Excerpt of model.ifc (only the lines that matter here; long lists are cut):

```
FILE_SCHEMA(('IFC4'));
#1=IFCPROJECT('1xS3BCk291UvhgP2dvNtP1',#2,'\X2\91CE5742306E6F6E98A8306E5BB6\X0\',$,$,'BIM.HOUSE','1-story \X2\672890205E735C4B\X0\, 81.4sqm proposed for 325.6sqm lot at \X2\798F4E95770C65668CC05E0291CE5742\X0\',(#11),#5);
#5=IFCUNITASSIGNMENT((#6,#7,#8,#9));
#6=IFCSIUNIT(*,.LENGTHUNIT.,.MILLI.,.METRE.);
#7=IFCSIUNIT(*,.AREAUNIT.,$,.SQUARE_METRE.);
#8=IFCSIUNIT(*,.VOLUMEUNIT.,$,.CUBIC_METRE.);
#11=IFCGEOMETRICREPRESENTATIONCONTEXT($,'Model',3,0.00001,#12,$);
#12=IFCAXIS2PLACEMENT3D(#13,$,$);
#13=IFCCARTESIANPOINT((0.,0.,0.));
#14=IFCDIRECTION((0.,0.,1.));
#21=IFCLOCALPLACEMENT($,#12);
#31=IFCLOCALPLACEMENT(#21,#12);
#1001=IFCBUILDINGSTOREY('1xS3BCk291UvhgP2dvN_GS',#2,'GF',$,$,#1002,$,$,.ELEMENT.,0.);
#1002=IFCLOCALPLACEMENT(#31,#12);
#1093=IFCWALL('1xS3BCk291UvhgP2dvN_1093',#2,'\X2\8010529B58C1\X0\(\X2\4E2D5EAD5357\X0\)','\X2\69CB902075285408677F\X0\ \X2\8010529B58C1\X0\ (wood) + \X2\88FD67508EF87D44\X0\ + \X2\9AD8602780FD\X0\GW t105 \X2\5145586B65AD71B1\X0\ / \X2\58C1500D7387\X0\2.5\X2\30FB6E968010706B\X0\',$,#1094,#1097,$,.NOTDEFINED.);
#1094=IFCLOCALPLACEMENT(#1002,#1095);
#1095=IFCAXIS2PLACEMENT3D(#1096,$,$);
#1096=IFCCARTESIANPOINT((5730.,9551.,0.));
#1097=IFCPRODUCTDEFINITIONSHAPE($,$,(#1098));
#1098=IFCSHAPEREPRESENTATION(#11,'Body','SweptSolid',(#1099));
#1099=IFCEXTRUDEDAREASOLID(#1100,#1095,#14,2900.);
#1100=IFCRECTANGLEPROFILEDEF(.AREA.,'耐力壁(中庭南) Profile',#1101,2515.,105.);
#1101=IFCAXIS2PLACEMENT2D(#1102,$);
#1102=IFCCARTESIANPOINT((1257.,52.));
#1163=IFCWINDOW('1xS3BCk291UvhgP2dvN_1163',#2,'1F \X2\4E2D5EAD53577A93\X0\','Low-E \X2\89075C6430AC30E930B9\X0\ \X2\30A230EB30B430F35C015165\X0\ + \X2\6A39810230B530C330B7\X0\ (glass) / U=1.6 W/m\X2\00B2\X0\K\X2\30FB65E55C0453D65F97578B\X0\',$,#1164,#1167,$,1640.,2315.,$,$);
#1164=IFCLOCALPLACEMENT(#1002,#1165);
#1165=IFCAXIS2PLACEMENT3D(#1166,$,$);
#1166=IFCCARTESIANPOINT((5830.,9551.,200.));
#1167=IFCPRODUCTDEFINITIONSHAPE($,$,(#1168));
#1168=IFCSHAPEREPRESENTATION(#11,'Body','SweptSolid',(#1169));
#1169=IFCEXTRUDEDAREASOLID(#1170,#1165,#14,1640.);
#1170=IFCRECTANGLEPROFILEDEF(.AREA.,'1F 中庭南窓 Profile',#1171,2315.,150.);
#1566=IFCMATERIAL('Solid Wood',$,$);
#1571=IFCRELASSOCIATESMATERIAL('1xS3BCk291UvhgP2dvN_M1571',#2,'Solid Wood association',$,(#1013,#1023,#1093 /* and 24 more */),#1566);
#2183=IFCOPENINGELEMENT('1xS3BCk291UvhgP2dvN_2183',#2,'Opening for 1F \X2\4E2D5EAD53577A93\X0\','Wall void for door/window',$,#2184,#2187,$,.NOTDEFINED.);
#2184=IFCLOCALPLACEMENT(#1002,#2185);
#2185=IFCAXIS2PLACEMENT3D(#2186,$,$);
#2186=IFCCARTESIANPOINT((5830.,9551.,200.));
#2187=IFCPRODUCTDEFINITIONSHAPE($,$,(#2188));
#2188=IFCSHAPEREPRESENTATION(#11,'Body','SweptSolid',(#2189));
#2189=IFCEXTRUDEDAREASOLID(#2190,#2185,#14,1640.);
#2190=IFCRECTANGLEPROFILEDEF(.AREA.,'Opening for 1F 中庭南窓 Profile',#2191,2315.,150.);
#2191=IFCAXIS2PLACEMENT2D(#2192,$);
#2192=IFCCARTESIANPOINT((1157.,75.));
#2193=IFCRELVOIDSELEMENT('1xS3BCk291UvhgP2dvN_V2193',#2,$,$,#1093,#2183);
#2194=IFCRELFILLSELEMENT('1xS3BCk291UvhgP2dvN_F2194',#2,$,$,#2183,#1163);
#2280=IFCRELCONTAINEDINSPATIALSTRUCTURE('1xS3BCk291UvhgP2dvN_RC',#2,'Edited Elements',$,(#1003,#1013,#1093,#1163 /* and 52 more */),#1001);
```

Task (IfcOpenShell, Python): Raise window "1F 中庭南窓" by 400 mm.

```python
import numpy as np
import ifcopenshell
import ifcopenshell.api.geometry
import ifcopenshell.util.placement
import ifcopenshell.util.unit

model = ifcopenshell.open("model.ifc")
unit_scale = ifcopenshell.util.unit.calculate_unit_scale(model)

window = model.by_guid("1xS3BCk291UvhgP2dvN_1163")
opening = window.FillsVoids[0].RelatingOpeningElement
dz = 0.4 / unit_scale

shift = np.array([0.0, 0.0, dz])
# The window is not placed relative to its opening, so move both.
for product in (opening, window):
    matrix = ifcopenshell.util.placement.get_local_placement(product.ObjectPlacement)
    matrix[:3, 3] += shift
    ifcopenshell.api.geometry.edit_object_placement(model, product=product, matrix=matrix, is_si=False)

print(f"moved by {dz * unit_scale:+.3f} m")

model.write("model_rev.ifc")
```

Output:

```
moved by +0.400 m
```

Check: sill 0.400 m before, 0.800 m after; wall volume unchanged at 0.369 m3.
